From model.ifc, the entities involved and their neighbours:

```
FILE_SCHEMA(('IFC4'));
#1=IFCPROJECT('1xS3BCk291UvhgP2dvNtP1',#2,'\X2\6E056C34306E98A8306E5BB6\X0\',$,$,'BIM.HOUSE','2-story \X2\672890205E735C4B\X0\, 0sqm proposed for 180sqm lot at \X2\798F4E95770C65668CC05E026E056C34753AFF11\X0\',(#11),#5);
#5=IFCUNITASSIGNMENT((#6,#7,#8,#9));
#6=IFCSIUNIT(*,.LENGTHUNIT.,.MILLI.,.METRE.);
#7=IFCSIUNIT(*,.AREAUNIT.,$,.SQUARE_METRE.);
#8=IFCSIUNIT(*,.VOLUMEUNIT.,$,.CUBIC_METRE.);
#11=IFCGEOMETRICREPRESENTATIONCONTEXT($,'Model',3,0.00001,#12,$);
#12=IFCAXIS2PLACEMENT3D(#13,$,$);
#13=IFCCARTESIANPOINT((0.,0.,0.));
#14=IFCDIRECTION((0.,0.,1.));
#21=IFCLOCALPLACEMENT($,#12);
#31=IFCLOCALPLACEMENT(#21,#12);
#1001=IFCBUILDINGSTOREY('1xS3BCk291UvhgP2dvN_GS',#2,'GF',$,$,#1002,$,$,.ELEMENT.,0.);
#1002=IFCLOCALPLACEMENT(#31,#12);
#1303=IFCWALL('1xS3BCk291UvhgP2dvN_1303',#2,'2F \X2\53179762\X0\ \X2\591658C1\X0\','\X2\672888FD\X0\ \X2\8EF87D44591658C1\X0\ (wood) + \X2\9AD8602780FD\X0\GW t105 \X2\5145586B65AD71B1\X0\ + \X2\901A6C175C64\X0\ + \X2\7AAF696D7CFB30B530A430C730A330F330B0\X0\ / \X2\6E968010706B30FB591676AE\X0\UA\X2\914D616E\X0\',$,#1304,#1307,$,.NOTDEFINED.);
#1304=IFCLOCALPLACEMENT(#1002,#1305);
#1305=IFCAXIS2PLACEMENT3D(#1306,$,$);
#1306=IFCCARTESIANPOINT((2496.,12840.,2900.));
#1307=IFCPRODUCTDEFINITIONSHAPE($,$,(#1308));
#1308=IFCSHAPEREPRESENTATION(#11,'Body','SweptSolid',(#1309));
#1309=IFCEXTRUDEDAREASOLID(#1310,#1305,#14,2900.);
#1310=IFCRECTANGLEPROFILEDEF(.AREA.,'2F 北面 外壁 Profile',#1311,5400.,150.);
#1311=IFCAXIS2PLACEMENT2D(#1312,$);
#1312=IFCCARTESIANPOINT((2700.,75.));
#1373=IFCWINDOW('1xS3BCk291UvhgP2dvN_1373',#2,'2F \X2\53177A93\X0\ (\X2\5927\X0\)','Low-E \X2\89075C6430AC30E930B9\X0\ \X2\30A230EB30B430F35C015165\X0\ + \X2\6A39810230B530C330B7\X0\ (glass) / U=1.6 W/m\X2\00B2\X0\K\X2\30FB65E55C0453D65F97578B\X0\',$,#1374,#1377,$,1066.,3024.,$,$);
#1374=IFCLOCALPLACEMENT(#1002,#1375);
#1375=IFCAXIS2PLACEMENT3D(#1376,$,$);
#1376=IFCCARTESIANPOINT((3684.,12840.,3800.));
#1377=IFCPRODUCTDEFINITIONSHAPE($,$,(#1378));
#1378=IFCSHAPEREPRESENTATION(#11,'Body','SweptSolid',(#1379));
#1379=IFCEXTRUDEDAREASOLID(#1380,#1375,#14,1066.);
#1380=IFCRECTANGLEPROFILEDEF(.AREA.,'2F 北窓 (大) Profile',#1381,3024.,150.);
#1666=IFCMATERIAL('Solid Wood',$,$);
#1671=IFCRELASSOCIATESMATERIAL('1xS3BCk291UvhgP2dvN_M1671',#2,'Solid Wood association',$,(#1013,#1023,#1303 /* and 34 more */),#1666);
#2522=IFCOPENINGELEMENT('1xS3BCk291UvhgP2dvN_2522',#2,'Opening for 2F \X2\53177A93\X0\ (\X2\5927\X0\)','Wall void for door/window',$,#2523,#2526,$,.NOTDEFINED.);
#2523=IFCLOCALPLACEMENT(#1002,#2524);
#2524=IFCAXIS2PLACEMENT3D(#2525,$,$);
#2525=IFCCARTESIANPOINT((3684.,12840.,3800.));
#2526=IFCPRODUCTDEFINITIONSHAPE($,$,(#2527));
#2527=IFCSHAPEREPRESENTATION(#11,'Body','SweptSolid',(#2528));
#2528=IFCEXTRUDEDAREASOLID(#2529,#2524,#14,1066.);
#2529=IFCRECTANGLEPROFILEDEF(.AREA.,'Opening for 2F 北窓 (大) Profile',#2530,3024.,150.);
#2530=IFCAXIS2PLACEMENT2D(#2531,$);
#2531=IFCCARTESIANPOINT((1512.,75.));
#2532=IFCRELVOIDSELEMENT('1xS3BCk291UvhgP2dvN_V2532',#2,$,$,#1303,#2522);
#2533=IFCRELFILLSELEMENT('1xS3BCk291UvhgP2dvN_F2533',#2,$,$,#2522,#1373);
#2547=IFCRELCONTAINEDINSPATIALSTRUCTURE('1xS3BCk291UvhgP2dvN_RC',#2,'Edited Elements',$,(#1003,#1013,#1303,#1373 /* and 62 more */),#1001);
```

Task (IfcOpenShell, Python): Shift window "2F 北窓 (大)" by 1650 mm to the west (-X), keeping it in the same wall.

```python
import ifcopenshell
import ifcopenshell.api.geometry
import ifcopenshell.util.placement
import ifcopenshell.util.unit

model = ifcopenshell.open("model.ifc")
unit_scale = ifcopenshell.util.unit.calculate_unit_scale(model)

window = model.by_guid("1xS3BCk291UvhgP2dvN_1373")
opening = window.FillsVoids[0].RelatingOpeningElement
wall = opening.VoidsElements[0].RelatingBuildingElement

wall_matrix = ifcopenshell.util.placement.get_local_placement(wall.ObjectPlacement)
shift = wall_matrix[:3, 0] * -1.65 / unit_scale
before = ifcopenshell.util.placement.get_local_placement(window.ObjectPlacement)[:3, 3].copy()

# The window is not placed relative to its opening, so move both.
for product in (opening, window):
    matrix = ifcopenshell.util.placement.get_local_placement(product.ObjectPlacement)
    matrix[:3, 3] += shift
    ifcopenshell.api.geometry.edit_object_placement(model, product=product, matrix=matrix, is_si=False)

after = ifcopenshell.util.placement.get_local_placement(window.ObjectPlacement)[:3, 3]
print("window moved by", (after - before).round(3) + 0.0)

model.write("model_rev.ifc")
```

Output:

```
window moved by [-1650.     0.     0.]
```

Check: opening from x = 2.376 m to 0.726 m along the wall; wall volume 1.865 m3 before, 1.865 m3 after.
